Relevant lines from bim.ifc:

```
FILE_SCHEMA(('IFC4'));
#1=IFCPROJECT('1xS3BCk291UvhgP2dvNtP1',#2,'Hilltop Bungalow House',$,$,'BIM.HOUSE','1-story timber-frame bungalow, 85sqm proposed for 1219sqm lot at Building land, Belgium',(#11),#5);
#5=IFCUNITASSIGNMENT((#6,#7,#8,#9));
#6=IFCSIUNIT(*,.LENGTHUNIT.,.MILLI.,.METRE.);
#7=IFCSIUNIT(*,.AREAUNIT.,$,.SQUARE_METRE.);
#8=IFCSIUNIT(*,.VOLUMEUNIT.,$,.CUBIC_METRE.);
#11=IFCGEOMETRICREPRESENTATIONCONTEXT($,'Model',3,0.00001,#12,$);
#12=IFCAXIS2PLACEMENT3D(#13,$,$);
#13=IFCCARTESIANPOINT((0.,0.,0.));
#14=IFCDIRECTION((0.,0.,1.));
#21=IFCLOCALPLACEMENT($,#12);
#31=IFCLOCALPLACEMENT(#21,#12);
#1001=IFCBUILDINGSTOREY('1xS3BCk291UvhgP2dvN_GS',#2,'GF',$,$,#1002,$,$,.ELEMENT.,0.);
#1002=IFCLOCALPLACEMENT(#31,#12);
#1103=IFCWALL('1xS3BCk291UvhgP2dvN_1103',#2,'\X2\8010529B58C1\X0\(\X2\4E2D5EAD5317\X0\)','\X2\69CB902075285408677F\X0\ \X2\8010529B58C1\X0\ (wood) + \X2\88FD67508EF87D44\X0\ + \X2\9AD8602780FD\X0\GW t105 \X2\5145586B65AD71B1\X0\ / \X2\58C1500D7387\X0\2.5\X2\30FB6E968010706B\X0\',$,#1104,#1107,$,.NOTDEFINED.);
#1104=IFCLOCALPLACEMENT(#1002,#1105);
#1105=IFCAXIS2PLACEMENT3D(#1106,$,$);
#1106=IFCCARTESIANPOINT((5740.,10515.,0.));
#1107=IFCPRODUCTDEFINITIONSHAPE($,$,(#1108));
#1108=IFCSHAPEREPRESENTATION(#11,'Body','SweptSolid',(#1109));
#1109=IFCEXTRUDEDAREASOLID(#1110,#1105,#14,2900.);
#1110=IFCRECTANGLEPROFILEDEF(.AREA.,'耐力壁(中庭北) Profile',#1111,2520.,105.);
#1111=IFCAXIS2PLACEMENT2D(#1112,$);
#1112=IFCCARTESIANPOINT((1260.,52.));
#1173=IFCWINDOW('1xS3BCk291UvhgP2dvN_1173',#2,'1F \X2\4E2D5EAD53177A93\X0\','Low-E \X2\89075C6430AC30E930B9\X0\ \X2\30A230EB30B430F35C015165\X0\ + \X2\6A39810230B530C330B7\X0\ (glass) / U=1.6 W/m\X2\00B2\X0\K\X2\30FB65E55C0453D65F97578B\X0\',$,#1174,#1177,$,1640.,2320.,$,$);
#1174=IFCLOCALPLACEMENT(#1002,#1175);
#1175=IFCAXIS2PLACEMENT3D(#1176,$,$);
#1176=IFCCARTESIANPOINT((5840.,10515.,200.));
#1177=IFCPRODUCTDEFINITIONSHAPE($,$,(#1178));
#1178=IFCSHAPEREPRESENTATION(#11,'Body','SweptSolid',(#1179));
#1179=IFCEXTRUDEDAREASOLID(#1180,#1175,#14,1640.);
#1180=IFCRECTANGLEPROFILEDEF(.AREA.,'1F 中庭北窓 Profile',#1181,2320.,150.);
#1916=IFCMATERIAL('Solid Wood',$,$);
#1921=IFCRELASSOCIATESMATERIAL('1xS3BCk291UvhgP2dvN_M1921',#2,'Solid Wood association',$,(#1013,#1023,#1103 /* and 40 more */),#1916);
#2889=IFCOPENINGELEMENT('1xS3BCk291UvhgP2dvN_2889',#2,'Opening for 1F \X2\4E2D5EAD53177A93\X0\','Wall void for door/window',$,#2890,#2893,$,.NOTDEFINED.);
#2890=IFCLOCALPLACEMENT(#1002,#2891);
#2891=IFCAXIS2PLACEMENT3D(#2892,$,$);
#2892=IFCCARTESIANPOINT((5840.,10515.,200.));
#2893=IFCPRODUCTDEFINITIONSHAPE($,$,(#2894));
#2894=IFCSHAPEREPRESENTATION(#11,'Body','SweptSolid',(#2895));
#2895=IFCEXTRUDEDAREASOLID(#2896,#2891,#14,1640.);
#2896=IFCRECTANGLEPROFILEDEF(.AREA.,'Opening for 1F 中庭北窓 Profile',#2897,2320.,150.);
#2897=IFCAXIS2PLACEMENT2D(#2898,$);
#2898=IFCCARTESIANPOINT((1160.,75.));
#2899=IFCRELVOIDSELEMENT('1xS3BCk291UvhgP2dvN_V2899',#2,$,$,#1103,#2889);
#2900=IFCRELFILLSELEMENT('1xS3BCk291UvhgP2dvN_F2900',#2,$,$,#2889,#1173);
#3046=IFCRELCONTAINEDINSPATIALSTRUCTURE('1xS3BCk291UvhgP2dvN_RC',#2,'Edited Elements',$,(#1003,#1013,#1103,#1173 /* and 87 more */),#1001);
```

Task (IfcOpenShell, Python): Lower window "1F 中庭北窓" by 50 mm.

```python
import numpy as np
import ifcopenshell
import ifcopenshell.api.geometry
import ifcopenshell.util.placement
import ifcopenshell.util.unit

model = ifcopenshell.open("bim.ifc")
unit_scale = ifcopenshell.util.unit.calculate_unit_scale(model)

window = model.by_guid("1xS3BCk291UvhgP2dvN_1173")
opening = window.FillsVoids[0].RelatingOpeningElement
dz = -50.0

shift = np.array([0.0, 0.0, dz])
# The window is not placed relative to its opening, so move both.
for product in (opening, window):
    matrix = ifcopenshell.util.placement.get_local_placement(product.ObjectPlacement)
    matrix[:3, 3] += shift
    ifcopenshell.api.geometry.edit_object_placement(model, product=product, matrix=matrix, is_si=False)

print(f"moved by {dz * unit_scale:+.3f} m")

model.write("bim_rev.ifc")
```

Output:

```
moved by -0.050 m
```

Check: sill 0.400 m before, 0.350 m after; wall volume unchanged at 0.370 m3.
